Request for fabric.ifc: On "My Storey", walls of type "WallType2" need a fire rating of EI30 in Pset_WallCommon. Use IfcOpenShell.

First a look at what the model holds.

```python
import ifcopenshell
import ifcopenshell.util.element

model = ifcopenshell.open("fabric.ifc")
print(model.schema)
storey = next(s for s in model.by_type("IfcBuildingStorey") if s.Name == "My Storey")
walls = [e for e in ifcopenshell.util.element.get_decomposition(storey) if e.is_a("IfcWall")]
seen = {}
for e in walls:
    element_type = ifcopenshell.util.element.get_type(e)
    key = (element_type.Name if element_type != e and element_type else None, ifcopenshell.util.element.get_pset(e, "Pset_WallCommon", "FireRating"))
    seen[key] = seen.get(key, 0) + 1
for (name, value), count in sorted(seen.items(), key=str):
    print(count, "x", name, "|", value)
```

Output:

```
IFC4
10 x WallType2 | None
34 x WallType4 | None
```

```python
import ifcopenshell
import ifcopenshell.api.pset
import ifcopenshell.util.element

model = ifcopenshell.open("fabric.ifc")

storey = next(s for s in model.by_type("IfcBuildingStorey") if s.Name == "My Storey")
walls = [e for e in ifcopenshell.util.element.get_decomposition(storey) if e.is_a("IfcWall")]

count = 0
for e in walls:
    element_type = ifcopenshell.util.element.get_type(e)
    if element_type in (None, e) or element_type.Name != "WallType2":
        continue
    # add_pset returns the element's existing set when there is one.
    pset = ifcopenshell.api.pset.add_pset(model, product=e, name="Pset_WallCommon")
    ifcopenshell.api.pset.edit_pset(model, pset=pset, properties={"FireRating": "EI30"})
    count += 1

print(count, "walls updated")

model.write("fabric_v2.ifc")
```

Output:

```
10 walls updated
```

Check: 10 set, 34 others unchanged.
